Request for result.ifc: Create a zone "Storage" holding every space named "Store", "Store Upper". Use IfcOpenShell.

First a look at what the model holds.

```python
import ifcopenshell

model = ifcopenshell.open("result.ifc")
print(model.schema)
seen = {}
for space in model.by_type("IfcSpace"):
    seen[space.LongName] = seen.get(space.LongName, 0) + 1
for name, count in sorted(seen.items(), key=str):
    print(count, "x", name)
print("zones:", [z.Name for z in model.by_type("IfcZone")][:20])
```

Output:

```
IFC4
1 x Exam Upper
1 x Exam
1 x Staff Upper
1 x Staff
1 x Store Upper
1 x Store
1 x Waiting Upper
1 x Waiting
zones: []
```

```python
import ifcopenshell
import ifcopenshell.api.group
import ifcopenshell.api.root

model = ifcopenshell.open("result.ifc")

names = {"Store", "Store Upper"}
spaces = [s for s in model.by_type("IfcSpace") if s.LongName in names]

zone = ifcopenshell.api.root.create_entity(model, ifc_class="IfcZone", name="Storage")
ifcopenshell.api.group.assign_group(model, products=spaces, group=zone)
print(len(spaces), "spaces in", zone.Name)

model.write("result-out.ifc")
```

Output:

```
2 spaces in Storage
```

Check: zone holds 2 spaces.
